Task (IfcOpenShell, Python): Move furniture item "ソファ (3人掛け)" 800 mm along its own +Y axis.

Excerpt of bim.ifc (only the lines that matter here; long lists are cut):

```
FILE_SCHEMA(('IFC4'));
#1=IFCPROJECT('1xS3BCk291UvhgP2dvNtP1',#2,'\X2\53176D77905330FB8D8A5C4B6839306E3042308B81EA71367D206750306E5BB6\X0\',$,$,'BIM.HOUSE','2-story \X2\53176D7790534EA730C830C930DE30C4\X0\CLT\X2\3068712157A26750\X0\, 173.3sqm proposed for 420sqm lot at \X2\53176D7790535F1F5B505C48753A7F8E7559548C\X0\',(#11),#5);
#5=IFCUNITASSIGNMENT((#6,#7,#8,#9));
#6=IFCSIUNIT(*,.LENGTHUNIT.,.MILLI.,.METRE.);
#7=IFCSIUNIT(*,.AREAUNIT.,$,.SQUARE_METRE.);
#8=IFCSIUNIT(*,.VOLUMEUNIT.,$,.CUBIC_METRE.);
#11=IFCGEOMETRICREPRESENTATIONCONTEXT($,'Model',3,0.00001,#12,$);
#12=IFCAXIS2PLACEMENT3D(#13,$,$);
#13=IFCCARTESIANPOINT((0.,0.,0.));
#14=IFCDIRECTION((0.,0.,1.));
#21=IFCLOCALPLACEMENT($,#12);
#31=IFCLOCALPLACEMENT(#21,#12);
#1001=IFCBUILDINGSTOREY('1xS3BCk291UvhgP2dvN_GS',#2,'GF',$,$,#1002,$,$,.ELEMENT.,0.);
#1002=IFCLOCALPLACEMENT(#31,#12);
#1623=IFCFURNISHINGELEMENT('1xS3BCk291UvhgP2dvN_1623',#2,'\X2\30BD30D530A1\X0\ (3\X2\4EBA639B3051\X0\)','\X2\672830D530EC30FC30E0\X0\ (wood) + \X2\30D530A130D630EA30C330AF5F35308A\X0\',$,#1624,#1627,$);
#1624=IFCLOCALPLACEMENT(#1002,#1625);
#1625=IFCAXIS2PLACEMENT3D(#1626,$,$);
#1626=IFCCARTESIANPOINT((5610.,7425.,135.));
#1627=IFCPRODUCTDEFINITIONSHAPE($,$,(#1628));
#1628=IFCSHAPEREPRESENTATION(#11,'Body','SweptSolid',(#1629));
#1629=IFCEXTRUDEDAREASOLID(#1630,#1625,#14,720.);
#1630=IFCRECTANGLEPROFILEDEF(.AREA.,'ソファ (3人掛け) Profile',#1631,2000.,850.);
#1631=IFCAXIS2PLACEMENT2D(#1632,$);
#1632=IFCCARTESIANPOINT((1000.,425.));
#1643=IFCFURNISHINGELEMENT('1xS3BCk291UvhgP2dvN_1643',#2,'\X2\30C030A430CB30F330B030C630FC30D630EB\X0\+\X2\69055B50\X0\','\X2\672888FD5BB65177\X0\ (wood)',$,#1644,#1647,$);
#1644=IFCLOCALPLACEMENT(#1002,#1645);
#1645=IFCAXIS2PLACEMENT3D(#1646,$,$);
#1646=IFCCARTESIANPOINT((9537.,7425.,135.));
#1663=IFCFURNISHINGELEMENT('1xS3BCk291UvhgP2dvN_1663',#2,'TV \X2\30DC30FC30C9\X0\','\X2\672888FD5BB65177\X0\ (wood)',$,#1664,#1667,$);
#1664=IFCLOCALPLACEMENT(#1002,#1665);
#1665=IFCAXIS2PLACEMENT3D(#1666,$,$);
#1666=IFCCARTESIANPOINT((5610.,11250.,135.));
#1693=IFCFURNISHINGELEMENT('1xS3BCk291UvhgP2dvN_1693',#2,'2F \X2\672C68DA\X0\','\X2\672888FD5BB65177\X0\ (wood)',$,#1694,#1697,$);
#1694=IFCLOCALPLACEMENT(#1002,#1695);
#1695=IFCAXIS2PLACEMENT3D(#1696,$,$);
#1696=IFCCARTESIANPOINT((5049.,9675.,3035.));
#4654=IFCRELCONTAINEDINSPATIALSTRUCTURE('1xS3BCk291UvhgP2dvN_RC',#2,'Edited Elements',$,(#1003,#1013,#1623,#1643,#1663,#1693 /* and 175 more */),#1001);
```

```python
import ifcopenshell
import ifcopenshell.api.geometry
import ifcopenshell.util.placement

model = ifcopenshell.open("bim.ifc")

item = model.by_guid("1xS3BCk291UvhgP2dvN_1623")
matrix = ifcopenshell.util.placement.get_local_placement(item.ObjectPlacement)
matrix[:3, 3] += matrix[:3, 1] * 800.0
ifcopenshell.api.geometry.edit_object_placement(model, product=item, matrix=matrix, is_si=False)

print(ifcopenshell.util.placement.get_local_placement(item.ObjectPlacement).round(3) + 0.0)

model.write("bim_updated.ifc")
```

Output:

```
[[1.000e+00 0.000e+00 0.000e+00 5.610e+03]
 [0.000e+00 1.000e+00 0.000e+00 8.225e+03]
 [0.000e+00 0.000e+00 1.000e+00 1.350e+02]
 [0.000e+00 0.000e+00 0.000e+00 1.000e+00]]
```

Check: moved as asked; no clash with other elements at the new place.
